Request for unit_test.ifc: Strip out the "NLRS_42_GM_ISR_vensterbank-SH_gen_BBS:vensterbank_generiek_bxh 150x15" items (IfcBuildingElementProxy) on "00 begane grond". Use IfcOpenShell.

First a look at what the model holds.

```python
import ifcopenshell
import ifcopenshell.util.element

model = ifcopenshell.open("unit_test.ifc")
print(model.schema)
storey = next(s for s in model.by_type("IfcBuildingStorey") if s.Name == "00 begane grond")
proxies = [e for e in ifcopenshell.util.element.get_decomposition(storey) if e.is_a("IfcBuildingElementProxy")]
seen = {}
for e in proxies:
    element_type = ifcopenshell.util.element.get_type(e)
    name = element_type.Name if element_type not in (None, e) else None
    seen[name] = seen.get(name, 0) + 1
for name, count in sorted(seen.items(), key=str):
    print(count, "x", name)
```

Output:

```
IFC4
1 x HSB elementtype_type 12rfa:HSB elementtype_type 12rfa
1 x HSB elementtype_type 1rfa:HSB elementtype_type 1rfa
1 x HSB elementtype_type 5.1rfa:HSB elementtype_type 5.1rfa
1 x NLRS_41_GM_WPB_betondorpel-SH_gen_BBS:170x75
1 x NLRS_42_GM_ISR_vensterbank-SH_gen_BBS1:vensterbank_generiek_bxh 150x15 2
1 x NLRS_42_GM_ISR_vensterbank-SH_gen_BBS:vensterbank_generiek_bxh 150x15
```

```python
import ifcopenshell
import ifcopenshell.api.root
import ifcopenshell.util.element

model = ifcopenshell.open("unit_test.ifc")

storey = next(s for s in model.by_type("IfcBuildingStorey") if s.Name == "00 begane grond")
proxies = [e for e in ifcopenshell.util.element.get_decomposition(storey) if e.is_a("IfcBuildingElementProxy")]
targets = [e for e in proxies if (t := ifcopenshell.util.element.get_type(e)) not in (None, e) and t.Name == "NLRS_42_GM_ISR_vensterbank-SH_gen_BBS:vensterbank_generiek_bxh 150x15"]

for e in targets:
    ifcopenshell.api.root.remove_product(model, product=e)
print(len(targets), "removed")

model.write("unit_test_edited.ifc")
```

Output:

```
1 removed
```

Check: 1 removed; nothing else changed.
